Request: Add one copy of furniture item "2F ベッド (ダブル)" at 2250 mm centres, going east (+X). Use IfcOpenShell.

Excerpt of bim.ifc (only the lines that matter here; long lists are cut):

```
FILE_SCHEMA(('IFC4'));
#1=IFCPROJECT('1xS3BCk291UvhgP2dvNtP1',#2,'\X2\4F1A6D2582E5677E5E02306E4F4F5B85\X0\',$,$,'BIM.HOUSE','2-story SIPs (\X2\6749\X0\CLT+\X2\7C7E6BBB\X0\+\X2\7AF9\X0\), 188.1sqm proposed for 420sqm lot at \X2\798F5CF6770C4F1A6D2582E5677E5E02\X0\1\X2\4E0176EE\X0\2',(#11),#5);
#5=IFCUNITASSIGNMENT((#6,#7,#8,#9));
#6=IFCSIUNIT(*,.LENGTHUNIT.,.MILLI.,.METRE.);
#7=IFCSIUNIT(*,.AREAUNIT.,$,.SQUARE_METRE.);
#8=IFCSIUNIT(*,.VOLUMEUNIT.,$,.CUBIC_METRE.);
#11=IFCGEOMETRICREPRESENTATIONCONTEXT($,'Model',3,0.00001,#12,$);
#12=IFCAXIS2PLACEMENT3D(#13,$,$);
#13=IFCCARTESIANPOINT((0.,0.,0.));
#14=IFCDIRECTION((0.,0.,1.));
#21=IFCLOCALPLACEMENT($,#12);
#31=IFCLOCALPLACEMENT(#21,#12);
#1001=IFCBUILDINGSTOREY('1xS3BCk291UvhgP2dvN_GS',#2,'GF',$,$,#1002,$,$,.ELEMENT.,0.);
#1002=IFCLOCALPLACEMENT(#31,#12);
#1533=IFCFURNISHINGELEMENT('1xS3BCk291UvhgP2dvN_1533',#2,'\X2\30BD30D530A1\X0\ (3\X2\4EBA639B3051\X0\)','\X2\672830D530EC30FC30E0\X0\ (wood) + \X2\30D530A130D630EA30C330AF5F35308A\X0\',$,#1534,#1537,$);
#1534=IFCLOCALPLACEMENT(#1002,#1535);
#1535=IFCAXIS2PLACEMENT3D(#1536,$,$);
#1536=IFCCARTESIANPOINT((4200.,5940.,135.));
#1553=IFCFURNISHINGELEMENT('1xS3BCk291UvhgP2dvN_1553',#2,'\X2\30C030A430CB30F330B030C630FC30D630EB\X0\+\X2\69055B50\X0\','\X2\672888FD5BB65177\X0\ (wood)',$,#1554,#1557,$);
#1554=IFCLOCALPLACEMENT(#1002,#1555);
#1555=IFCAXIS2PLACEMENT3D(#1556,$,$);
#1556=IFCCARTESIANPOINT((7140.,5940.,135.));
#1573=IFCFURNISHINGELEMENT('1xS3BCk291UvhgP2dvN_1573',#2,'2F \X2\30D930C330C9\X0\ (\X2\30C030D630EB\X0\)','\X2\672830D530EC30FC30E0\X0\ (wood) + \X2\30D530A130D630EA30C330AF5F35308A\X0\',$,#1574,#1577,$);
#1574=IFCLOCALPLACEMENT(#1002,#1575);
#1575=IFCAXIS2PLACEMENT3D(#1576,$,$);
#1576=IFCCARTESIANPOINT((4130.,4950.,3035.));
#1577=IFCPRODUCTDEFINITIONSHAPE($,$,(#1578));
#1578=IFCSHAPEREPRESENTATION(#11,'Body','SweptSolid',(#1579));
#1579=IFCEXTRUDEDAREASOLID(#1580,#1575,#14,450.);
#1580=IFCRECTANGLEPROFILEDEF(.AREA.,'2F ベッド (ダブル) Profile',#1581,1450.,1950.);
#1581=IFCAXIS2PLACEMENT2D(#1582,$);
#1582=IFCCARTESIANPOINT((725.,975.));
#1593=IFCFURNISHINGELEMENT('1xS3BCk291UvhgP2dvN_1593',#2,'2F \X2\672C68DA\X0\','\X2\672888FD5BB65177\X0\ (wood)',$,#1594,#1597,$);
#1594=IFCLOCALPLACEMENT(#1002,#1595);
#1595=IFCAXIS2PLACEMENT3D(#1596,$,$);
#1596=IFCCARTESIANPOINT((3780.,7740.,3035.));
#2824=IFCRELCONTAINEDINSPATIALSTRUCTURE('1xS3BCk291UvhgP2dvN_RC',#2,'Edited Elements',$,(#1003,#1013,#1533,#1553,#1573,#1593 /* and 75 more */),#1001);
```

```python
import numpy as np
import ifcopenshell
import ifcopenshell.api.geometry
import ifcopenshell.api.root
import ifcopenshell.util.element
import ifcopenshell.util.placement
import ifcopenshell.util.unit

model = ifcopenshell.open("bim.ifc")
unit_scale = ifcopenshell.util.unit.calculate_unit_scale(model)


def reuse_history(source, copy):
    """copy_class also copies each property set's owner history, people and application; keep the originals."""
    for rel in copy.IsDefinedBy:
        if rel.is_a("IfcRelDefinesByProperties") and (history := rel.RelatingPropertyDefinition.OwnerHistory):
            rel.RelatingPropertyDefinition.OwnerHistory = source.OwnerHistory
            ifcopenshell.util.element.remove_deep2(model, history)


source = model.by_guid("1xS3BCk291UvhgP2dvN_1573")
base = ifcopenshell.util.placement.get_local_placement(source.ObjectPlacement)
step = np.array([1.0, 0.0, 0.0]) * 2.25 / unit_scale

for i in range(1, 2):
    copy = ifcopenshell.api.root.copy_class(model, product=source)
    copy.Representation = ifcopenshell.util.element.copy_deep(
        model, source.Representation, exclude=["IfcGeometricRepresentationContext", "IfcRepresentationMap"]
    )
    reuse_history(source, copy)
    matrix = base.copy()
    matrix[:3, 3] += i * step
    print("added at", matrix[:3, 3].round(3) + 0.0)
    ifcopenshell.api.geometry.edit_object_placement(model, product=copy, matrix=matrix, is_si=False)

model.write("bim_v2.ifc")
```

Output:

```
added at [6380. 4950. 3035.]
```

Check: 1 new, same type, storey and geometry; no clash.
